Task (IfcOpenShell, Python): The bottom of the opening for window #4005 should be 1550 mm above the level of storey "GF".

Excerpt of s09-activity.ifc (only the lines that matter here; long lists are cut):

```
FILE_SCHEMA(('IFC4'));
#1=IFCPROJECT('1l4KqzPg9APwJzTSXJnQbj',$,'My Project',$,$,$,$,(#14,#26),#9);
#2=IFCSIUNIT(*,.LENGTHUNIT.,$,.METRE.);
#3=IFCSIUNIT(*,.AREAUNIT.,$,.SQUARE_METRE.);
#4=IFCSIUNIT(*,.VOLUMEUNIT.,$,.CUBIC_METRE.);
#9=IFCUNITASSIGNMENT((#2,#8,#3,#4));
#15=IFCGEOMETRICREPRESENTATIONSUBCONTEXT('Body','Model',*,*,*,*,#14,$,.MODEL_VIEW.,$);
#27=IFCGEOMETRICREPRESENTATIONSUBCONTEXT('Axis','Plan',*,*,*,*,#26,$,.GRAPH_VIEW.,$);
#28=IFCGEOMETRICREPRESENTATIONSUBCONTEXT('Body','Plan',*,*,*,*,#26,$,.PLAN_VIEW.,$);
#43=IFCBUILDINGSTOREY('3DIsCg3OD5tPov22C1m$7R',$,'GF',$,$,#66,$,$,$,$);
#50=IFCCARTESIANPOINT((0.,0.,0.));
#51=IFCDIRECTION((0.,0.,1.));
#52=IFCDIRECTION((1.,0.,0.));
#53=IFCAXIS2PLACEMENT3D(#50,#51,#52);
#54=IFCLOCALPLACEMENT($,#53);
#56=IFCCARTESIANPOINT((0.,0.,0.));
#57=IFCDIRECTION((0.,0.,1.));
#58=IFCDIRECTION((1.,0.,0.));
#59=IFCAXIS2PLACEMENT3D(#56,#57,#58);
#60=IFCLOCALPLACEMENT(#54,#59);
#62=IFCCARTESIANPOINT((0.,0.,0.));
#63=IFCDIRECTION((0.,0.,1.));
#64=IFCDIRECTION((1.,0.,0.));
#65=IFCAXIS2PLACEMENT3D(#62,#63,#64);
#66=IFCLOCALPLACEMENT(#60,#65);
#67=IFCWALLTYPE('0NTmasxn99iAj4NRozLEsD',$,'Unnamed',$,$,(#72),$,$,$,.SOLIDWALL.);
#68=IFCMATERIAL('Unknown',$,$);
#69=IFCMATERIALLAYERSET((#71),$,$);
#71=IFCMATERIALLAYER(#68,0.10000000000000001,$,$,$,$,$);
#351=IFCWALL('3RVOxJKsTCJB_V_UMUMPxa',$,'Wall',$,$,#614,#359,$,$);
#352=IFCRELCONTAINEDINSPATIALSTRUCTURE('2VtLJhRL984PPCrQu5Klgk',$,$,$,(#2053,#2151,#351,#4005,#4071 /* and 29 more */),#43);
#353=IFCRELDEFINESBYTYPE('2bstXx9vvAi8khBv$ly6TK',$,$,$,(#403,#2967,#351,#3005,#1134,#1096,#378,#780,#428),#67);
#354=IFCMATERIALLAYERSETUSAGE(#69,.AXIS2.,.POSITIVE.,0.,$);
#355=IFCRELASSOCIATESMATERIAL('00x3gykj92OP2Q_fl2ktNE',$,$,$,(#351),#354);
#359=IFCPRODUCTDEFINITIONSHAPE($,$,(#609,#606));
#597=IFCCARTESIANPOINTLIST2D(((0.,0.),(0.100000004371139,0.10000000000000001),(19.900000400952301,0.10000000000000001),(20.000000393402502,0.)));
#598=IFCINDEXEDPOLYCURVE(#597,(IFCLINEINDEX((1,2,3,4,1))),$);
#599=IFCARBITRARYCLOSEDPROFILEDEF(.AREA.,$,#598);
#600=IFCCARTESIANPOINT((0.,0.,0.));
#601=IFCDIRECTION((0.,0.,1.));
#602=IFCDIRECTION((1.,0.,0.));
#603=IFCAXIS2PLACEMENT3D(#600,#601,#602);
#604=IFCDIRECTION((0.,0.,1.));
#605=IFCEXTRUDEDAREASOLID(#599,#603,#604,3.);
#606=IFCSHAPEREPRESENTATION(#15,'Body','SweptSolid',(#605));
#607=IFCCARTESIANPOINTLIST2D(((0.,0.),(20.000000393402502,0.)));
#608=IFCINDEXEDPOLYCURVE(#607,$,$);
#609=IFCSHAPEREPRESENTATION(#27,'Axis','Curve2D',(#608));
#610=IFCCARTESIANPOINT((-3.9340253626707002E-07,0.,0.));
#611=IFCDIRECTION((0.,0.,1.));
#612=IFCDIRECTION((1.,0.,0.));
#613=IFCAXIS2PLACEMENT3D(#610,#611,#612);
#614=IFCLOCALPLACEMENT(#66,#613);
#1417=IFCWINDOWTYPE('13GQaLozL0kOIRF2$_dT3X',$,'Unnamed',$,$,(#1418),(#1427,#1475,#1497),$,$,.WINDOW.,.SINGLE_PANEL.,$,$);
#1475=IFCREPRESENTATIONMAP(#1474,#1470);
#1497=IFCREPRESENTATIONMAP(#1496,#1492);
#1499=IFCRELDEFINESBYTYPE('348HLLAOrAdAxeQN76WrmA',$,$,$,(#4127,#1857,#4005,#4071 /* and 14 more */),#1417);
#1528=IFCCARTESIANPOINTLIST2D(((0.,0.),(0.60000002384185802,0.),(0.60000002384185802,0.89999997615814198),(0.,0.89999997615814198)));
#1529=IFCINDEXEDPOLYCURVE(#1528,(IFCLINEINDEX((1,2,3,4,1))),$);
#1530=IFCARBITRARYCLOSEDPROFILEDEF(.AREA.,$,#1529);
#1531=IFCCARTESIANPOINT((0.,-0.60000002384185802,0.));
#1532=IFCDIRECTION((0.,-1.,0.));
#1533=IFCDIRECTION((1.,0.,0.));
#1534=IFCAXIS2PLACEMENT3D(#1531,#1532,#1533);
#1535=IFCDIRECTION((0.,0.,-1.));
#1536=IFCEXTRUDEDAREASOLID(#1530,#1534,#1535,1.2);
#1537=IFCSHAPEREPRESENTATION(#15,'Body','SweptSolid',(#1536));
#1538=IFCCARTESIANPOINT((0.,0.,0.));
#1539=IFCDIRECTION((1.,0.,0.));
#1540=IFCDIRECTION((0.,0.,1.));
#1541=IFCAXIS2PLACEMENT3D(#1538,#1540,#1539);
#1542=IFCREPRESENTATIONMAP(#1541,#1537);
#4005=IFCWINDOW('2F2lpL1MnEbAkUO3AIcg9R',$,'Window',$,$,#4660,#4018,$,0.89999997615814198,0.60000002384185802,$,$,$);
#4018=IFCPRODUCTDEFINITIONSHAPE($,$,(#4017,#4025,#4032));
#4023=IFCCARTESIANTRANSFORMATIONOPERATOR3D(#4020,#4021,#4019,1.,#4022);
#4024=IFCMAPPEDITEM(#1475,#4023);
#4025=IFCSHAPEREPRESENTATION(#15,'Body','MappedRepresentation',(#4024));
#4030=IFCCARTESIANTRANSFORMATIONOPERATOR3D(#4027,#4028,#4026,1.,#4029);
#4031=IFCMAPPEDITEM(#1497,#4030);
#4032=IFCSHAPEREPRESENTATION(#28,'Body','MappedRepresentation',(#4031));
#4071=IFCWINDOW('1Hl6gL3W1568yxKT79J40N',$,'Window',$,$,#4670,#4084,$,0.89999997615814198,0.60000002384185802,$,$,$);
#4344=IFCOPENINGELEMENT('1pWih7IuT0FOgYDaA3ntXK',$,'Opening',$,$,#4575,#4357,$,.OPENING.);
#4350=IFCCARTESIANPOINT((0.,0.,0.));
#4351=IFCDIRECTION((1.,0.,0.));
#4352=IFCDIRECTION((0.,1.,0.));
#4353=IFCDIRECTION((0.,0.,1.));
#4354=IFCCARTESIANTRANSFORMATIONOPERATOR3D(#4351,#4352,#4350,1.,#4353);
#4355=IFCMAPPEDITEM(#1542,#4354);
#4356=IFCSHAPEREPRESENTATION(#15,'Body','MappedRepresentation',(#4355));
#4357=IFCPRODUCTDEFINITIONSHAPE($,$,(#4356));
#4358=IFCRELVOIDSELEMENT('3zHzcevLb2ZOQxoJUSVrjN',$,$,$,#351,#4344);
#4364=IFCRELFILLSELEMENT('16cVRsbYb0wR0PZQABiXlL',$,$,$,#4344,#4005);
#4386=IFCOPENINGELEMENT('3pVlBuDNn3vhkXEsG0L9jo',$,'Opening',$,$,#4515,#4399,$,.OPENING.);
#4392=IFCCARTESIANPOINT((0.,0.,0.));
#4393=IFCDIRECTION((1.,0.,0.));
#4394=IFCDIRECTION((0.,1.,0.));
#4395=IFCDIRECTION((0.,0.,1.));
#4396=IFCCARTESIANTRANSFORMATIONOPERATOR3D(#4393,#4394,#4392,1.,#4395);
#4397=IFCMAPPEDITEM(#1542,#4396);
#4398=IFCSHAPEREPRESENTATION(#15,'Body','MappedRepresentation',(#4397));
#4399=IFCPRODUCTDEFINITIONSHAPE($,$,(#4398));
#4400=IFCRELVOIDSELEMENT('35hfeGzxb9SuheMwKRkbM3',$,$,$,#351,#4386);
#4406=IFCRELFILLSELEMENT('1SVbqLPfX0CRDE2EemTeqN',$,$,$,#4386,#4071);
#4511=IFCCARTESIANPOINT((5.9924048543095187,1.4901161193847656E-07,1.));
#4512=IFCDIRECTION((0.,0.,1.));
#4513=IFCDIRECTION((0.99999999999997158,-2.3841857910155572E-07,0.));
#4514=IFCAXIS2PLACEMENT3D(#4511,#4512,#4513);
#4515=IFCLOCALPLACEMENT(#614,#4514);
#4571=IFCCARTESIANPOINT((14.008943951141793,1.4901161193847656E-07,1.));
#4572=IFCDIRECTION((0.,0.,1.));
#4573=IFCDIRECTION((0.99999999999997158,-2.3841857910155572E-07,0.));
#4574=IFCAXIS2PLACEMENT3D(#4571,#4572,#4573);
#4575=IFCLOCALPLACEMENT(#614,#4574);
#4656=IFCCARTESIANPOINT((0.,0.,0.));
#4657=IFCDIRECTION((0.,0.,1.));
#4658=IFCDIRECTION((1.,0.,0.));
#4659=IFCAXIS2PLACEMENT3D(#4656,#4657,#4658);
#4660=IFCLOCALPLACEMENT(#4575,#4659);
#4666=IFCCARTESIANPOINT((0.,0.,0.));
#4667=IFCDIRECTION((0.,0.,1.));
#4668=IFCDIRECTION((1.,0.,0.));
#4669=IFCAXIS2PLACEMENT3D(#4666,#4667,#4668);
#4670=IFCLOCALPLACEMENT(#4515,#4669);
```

```python
import numpy as np
import ifcopenshell
import ifcopenshell.api.geometry
import ifcopenshell.geom
import ifcopenshell.util.element
import ifcopenshell.util.placement
import ifcopenshell.util.shape
import ifcopenshell.util.unit

model = ifcopenshell.open("s09-activity.ifc")
unit_scale = ifcopenshell.util.unit.calculate_unit_scale(model)

window = model.by_id(4005)
opening = window.FillsVoids[0].RelatingOpeningElement
storey = ifcopenshell.util.element.get_container(window, ifc_class="IfcBuildingStorey")
level = ifcopenshell.util.placement.get_local_placement(storey.ObjectPlacement)[2, 3]

# The opening's origin need not be at the sill, so measure its lowest point.
shape = ifcopenshell.geom.create_shape(ifcopenshell.geom.settings(), opening)
bottom = ifcopenshell.util.shape.get_shape_bottom_elevation(shape, shape.geometry) / unit_scale
dz = level + 1.55 / unit_scale - bottom

shift = np.array([0.0, 0.0, dz])
# The window is placed relative to its opening, so it follows when the opening moves.
matrix = ifcopenshell.util.placement.get_local_placement(opening.ObjectPlacement)
matrix[:3, 3] += shift
ifcopenshell.api.geometry.edit_object_placement(
    model, product=opening, matrix=matrix, is_si=False, should_transform_children=True
)

print(f"moved by {dz * unit_scale:+.3f} m")

model.write("s09-activity_rev.ifc")
```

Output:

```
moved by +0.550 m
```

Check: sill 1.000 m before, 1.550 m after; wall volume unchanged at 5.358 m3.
